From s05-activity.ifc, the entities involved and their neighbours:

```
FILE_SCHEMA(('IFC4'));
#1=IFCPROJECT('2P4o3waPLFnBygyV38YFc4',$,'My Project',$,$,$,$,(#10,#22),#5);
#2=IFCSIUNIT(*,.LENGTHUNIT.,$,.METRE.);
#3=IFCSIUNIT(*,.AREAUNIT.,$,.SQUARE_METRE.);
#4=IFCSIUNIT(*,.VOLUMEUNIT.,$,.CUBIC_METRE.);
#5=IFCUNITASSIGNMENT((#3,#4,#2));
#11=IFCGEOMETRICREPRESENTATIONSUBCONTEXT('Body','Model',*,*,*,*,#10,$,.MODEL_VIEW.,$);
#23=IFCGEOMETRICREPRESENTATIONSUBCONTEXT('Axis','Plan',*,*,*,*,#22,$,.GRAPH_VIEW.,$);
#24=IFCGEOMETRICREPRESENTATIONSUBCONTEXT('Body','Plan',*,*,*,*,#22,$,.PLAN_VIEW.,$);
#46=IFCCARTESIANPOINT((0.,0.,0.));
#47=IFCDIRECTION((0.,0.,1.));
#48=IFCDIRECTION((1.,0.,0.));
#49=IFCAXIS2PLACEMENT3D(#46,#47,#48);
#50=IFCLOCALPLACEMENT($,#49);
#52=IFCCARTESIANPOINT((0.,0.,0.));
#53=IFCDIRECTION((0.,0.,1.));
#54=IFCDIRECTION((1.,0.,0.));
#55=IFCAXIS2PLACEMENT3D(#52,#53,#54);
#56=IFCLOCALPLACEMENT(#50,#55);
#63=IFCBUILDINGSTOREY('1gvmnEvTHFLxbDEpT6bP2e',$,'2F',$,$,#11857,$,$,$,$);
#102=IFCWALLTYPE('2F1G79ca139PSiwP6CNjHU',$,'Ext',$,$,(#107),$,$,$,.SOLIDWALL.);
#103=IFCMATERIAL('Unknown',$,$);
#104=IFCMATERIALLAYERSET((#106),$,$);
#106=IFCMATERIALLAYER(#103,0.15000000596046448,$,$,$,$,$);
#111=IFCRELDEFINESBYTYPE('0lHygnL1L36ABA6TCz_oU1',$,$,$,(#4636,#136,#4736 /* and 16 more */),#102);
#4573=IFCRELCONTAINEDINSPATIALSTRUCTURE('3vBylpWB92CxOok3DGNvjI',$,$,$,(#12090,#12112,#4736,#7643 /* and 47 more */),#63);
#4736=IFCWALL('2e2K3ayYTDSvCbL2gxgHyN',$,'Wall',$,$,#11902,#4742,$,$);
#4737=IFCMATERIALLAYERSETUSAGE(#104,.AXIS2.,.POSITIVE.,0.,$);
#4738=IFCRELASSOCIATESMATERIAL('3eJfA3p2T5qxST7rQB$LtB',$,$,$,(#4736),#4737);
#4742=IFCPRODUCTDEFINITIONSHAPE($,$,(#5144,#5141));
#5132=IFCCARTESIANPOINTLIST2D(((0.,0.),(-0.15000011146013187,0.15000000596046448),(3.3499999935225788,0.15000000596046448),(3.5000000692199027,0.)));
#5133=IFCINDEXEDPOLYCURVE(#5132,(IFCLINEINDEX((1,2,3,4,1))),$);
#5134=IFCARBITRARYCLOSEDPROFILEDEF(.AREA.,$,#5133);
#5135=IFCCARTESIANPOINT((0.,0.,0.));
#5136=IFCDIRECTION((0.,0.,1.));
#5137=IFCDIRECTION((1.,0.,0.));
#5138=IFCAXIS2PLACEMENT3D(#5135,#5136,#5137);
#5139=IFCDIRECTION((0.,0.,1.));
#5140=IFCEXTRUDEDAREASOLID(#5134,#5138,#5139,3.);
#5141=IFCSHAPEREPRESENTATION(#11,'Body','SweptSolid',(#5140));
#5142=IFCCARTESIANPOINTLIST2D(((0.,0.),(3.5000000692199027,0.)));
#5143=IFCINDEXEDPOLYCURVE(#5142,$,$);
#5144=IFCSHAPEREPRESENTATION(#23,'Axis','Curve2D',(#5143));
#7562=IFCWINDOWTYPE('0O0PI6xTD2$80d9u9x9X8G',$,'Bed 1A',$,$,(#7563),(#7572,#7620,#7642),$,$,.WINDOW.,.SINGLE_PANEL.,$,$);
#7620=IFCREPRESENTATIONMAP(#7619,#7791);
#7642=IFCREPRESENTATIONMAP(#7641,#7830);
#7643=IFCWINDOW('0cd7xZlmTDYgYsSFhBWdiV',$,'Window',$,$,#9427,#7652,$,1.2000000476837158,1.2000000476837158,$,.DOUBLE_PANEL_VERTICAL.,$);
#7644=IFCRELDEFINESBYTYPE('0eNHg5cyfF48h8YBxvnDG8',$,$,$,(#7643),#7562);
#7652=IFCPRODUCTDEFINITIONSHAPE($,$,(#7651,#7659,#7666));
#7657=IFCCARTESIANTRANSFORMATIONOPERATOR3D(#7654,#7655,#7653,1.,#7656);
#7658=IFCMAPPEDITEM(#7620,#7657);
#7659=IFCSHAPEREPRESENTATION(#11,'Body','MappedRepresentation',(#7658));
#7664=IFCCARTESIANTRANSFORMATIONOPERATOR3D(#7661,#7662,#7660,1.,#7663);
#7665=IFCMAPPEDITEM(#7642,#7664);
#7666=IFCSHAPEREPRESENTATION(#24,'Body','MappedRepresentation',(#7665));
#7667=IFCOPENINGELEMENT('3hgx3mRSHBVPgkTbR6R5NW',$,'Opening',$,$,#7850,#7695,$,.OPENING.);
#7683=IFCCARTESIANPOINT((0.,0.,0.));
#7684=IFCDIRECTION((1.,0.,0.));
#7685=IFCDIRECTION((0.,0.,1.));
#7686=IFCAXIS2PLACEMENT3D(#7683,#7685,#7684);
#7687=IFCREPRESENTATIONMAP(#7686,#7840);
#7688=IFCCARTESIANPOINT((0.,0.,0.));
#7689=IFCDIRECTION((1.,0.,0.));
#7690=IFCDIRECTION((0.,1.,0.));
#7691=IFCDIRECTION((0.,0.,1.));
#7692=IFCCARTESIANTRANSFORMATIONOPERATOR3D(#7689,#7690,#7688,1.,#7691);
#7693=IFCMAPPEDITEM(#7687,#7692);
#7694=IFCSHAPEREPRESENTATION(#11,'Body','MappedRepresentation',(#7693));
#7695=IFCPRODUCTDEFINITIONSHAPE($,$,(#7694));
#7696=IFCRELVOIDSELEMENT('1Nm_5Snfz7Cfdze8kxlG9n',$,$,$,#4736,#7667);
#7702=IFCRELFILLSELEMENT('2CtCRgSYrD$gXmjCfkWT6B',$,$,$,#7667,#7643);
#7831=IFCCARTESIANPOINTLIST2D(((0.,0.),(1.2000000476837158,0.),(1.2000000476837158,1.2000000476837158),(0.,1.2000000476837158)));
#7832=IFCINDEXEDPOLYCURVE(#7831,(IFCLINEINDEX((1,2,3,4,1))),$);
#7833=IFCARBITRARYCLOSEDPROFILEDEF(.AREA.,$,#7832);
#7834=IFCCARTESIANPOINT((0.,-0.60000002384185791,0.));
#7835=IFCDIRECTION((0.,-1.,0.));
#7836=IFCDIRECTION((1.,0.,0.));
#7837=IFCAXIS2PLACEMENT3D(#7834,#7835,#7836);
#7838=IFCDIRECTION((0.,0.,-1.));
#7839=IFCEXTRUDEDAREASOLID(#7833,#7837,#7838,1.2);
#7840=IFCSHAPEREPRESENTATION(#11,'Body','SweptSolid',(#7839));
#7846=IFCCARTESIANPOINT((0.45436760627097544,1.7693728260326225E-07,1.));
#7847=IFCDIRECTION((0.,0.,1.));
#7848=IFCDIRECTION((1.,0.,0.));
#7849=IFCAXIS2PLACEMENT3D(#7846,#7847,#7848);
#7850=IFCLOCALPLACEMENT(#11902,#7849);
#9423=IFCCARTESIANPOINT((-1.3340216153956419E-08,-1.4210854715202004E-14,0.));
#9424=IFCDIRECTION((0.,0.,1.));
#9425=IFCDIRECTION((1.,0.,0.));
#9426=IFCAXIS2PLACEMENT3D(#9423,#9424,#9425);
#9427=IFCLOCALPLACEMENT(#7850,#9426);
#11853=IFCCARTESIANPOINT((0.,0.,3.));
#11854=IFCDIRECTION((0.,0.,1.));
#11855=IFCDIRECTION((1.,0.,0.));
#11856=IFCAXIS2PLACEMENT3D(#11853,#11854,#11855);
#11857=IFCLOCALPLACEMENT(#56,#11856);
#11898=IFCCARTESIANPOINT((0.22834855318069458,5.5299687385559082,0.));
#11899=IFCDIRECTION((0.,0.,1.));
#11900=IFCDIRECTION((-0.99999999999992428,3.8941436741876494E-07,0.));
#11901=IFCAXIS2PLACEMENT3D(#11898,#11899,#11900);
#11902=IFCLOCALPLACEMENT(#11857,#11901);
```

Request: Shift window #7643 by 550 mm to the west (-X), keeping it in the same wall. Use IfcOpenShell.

```python
import ifcopenshell
import ifcopenshell.api.geometry
import ifcopenshell.util.placement
import ifcopenshell.util.unit

model = ifcopenshell.open("s05-activity.ifc")
unit_scale = ifcopenshell.util.unit.calculate_unit_scale(model)

window = model.by_guid("0cd7xZlmTDYgYsSFhBWdiV")
opening = window.FillsVoids[0].RelatingOpeningElement
wall = opening.VoidsElements[0].RelatingBuildingElement

wall_matrix = ifcopenshell.util.placement.get_local_placement(wall.ObjectPlacement)
shift = wall_matrix[:3, 0] * 0.55 / unit_scale
before = ifcopenshell.util.placement.get_local_placement(window.ObjectPlacement)[:3, 3].copy()

# The window is placed relative to its opening, so it follows when the opening moves.
matrix = ifcopenshell.util.placement.get_local_placement(opening.ObjectPlacement)
matrix[:3, 3] += shift
ifcopenshell.api.geometry.edit_object_placement(
    model, product=opening, matrix=matrix, is_si=False, should_transform_children=True
)

after = ifcopenshell.util.placement.get_local_placement(window.ObjectPlacement)[:3, 3]
print("window moved by", (after - before).round(3) + 0.0)

model.write("s05-activity-out.ifc")
```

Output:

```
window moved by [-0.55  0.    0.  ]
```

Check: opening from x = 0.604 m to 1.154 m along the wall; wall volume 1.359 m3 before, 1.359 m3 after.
